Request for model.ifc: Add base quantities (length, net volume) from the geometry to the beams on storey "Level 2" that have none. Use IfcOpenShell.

First a look at what the model holds.

```python
import ifcopenshell
import ifcopenshell.util.element
import ifcopenshell.util.unit

model = ifcopenshell.open("model.ifc")
print(model.schema)
for unit_type in ("LENGTHUNIT", "AREAUNIT", "VOLUMEUNIT"):
    print(unit_type, ifcopenshell.util.unit.calculate_unit_scale(model, unit_type))
storey = next(s for s in model.by_type("IfcBuildingStorey") if s.Name == "Level 2")
beams = [e for e in ifcopenshell.util.element.get_decomposition(storey) if e.is_a("IfcBeam")]
for e in sorted(beams, key=lambda e: e.id()):
    print(e.id(), e.is_a(), e.Name, list(ifcopenshell.util.element.get_psets(e, qtos_only=True)), sep=" | ")
```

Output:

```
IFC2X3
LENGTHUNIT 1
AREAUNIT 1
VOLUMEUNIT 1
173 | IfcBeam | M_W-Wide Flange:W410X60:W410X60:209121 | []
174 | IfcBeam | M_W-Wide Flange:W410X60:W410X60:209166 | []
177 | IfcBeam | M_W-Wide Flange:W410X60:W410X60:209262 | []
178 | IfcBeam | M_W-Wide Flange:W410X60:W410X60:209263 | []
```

```python
import ifcopenshell
import ifcopenshell.api.pset
import ifcopenshell.geom
import ifcopenshell.util.element
import ifcopenshell.util.shape
import ifcopenshell.util.unit

model = ifcopenshell.open("model.ifc")
unit_scale = ifcopenshell.util.unit.calculate_unit_scale(model)
volume_scale = ifcopenshell.util.unit.calculate_unit_scale(model, "VOLUMEUNIT")
settings = ifcopenshell.geom.settings()

storey = next(s for s in model.by_type("IfcBuildingStorey") if s.Name == "Level 2")
beams = [e for e in ifcopenshell.util.element.get_decomposition(storey) if e.is_a("IfcBeam")]

for e in sorted(beams, key=lambda e: e.id()):
    if ifcopenshell.util.element.get_psets(e, qtos_only=True, should_inherit=False):
        continue
    # Geometry comes back in metres, in the element's own axes.
    shape = ifcopenshell.geom.create_shape(settings, e)
    values = {
        "Length": ifcopenshell.util.shape.get_max_xyz(shape.geometry) / unit_scale,
        "NetVolume": ifcopenshell.util.shape.get_volume(shape.geometry) / volume_scale,
    }
    qto = ifcopenshell.api.pset.add_qto(model, product=e, name="BaseQuantities")
    ifcopenshell.api.pset.edit_qto(model, qto=qto, properties=values)
    print(e.id(), {k: round(v, 3) for k, v in values.items()})

model.write("model_edited.ifc")
```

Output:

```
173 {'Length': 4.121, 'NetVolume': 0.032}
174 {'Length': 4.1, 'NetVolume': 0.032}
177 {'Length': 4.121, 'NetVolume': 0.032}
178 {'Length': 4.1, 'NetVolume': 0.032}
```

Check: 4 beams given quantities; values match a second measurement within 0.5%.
